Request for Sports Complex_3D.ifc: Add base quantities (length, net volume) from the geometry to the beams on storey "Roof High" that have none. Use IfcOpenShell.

First a look at what the model holds.

```python
import ifcopenshell
import ifcopenshell.util.element
import ifcopenshell.util.unit

model = ifcopenshell.open("Sports Complex_3D.ifc")
print(model.schema)
for unit_type in ("LENGTHUNIT", "AREAUNIT", "VOLUMEUNIT"):
    print(unit_type, ifcopenshell.util.unit.calculate_unit_scale(model, unit_type))
storey = next(s for s in model.by_type("IfcBuildingStorey") if s.Name == "Roof High")
beams = [e for e in ifcopenshell.util.element.get_decomposition(storey) if e.is_a("IfcBeam")]
for e in sorted(beams, key=lambda e: e.id()):
    print(e.id(), e.is_a(), e.Name, list(ifcopenshell.util.element.get_psets(e, qtos_only=True)), sep=" | ")
```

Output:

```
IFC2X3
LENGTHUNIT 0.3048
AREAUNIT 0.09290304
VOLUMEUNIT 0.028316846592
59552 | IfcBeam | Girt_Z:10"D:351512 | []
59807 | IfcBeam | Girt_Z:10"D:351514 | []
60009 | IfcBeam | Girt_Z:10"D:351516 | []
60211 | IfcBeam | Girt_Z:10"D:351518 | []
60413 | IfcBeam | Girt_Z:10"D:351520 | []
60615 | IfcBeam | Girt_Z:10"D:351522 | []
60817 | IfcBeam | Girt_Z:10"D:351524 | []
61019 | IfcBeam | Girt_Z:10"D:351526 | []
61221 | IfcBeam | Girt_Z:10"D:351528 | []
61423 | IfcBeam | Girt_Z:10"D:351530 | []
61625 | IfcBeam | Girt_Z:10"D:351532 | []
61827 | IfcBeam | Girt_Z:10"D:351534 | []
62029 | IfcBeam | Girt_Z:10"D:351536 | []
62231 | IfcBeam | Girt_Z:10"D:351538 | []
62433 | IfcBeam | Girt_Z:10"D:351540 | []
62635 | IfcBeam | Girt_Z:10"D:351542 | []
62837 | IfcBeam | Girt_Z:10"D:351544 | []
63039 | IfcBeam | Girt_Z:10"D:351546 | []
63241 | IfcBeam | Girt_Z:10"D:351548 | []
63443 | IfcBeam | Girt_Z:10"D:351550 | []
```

```python
import ifcopenshell
import ifcopenshell.api.pset
import ifcopenshell.geom
import ifcopenshell.util.element
import ifcopenshell.util.shape
import ifcopenshell.util.unit

model = ifcopenshell.open("Sports Complex_3D.ifc")
unit_scale = ifcopenshell.util.unit.calculate_unit_scale(model)
volume_scale = ifcopenshell.util.unit.calculate_unit_scale(model, "VOLUMEUNIT")
settings = ifcopenshell.geom.settings()

storey = next(s for s in model.by_type("IfcBuildingStorey") if s.Name == "Roof High")
beams = [e for e in ifcopenshell.util.element.get_decomposition(storey) if e.is_a("IfcBeam")]

for e in sorted(beams, key=lambda e: e.id()):
    if ifcopenshell.util.element.get_psets(e, qtos_only=True, should_inherit=False):
        continue
    # Geometry comes back in metres, in the element's own axes.
    shape = ifcopenshell.geom.create_shape(settings, e)
    values = {
        "Length": ifcopenshell.util.shape.get_max_xyz(shape.geometry) / unit_scale,
        "NetVolume": ifcopenshell.util.shape.get_volume(shape.geometry) / volume_scale,
    }
    qto = ifcopenshell.api.pset.add_qto(model, product=e, name="BaseQuantities")
    ifcopenshell.api.pset.edit_qto(model, qto=qto, properties=values)
    print(e.id(), {k: round(v, 3) for k, v in values.items()})

model.write("Sports Complex_3D_rev.ifc")
```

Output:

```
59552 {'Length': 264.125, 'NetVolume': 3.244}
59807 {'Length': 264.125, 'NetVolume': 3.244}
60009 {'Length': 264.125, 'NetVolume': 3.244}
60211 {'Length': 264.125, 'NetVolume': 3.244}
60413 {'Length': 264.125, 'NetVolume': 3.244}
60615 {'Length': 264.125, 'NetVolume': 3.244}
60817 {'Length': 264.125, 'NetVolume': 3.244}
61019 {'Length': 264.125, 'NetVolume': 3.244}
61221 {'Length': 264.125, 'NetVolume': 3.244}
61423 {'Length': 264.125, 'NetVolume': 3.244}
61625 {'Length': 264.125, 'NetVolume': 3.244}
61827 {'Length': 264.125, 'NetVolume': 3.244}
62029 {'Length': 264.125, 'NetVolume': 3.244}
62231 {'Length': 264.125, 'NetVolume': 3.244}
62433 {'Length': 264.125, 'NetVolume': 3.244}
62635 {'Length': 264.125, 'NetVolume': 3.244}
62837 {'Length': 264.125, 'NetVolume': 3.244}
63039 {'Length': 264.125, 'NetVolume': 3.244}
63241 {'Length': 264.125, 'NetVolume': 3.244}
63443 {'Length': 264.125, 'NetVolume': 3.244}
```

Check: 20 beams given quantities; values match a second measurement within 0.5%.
